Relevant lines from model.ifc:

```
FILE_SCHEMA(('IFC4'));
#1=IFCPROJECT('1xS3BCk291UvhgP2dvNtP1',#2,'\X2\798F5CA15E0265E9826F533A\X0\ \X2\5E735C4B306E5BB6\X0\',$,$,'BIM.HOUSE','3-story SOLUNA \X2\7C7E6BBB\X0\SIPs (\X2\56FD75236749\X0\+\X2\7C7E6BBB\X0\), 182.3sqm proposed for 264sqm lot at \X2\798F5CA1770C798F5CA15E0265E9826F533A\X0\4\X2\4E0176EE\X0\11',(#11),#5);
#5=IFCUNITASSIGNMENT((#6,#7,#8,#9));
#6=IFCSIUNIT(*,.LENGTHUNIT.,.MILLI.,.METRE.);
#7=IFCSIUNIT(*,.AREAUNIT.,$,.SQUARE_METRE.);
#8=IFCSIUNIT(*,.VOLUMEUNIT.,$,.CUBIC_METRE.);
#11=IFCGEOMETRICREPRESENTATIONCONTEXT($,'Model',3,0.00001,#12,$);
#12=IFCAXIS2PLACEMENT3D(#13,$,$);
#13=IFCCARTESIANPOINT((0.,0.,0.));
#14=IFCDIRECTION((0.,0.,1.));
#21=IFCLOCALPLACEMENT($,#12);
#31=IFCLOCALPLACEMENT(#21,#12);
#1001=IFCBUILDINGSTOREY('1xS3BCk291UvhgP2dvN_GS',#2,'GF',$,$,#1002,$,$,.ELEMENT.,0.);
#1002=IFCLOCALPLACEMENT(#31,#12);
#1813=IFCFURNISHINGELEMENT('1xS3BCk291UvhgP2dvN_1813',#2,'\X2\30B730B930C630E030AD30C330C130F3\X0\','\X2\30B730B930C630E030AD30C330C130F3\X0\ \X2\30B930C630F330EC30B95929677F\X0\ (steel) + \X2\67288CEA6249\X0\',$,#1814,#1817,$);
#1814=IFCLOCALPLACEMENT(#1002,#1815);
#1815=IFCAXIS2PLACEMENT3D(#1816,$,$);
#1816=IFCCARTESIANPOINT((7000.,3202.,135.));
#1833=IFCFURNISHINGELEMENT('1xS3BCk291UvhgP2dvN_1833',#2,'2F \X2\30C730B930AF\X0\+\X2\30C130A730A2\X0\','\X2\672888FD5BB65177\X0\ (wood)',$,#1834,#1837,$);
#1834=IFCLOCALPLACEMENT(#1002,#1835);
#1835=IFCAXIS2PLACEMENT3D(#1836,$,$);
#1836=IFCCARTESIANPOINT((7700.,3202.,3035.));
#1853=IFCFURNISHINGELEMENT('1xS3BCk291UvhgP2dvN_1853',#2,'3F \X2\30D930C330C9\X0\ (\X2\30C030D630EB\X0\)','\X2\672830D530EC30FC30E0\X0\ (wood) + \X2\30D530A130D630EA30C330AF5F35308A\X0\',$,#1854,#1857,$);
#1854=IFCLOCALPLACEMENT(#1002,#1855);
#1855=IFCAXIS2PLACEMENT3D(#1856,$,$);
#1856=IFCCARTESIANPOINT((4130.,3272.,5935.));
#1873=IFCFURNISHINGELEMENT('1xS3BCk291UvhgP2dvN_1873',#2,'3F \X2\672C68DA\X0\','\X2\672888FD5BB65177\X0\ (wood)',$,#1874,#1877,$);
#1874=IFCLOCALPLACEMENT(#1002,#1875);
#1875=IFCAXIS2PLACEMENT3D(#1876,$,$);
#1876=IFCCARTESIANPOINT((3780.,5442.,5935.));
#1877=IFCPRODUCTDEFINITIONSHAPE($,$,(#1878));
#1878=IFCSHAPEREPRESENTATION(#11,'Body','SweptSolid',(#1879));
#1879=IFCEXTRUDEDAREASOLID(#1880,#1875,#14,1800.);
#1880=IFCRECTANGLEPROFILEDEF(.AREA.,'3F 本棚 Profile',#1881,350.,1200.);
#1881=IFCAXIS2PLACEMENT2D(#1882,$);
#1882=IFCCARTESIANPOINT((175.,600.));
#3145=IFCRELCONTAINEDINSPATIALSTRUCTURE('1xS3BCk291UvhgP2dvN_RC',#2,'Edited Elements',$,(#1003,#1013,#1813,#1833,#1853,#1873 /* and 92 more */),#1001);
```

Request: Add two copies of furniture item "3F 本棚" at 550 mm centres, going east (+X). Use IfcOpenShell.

```python
import numpy as np
import ifcopenshell
import ifcopenshell.api.geometry
import ifcopenshell.api.root
import ifcopenshell.util.element
import ifcopenshell.util.placement

model = ifcopenshell.open("model.ifc")


def reuse_history(source, copy):
    """copy_class also copies each property set's owner history, people and application; keep the originals."""
    for rel in copy.IsDefinedBy:
        if rel.is_a("IfcRelDefinesByProperties") and (history := rel.RelatingPropertyDefinition.OwnerHistory):
            rel.RelatingPropertyDefinition.OwnerHistory = source.OwnerHistory
            ifcopenshell.util.element.remove_deep2(model, history)


source = model.by_id(1873)
base = ifcopenshell.util.placement.get_local_placement(source.ObjectPlacement)
step = np.array([1.0, 0.0, 0.0]) * 550.0

for i in range(1, 3):
    copy = ifcopenshell.api.root.copy_class(model, product=source)
    copy.Representation = ifcopenshell.util.element.copy_deep(
        model, source.Representation, exclude=["IfcGeometricRepresentationContext", "IfcRepresentationMap"]
    )
    reuse_history(source, copy)
    matrix = base.copy()
    matrix[:3, 3] += i * step
    print("added at", matrix[:3, 3].round(3) + 0.0)
    ifcopenshell.api.geometry.edit_object_placement(model, product=copy, matrix=matrix, is_si=False)

model.write("model_edited.ifc")
```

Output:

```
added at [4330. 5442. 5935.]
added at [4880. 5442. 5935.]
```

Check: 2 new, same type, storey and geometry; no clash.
